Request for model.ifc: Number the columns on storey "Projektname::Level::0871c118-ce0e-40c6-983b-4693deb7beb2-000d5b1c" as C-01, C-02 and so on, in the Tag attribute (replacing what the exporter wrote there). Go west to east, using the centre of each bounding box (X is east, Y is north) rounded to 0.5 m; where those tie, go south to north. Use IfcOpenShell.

First a look at what the model holds.

```python
import ifcopenshell
import ifcopenshell.util.element
import ifcopenshell.util.placement

model = ifcopenshell.open("model.ifc")
print(model.schema)
storey = next(s for s in model.by_type("IfcBuildingStorey") if s.Name == "Projektname::Level::0871c118-ce0e-40c6-983b-4693deb7beb2-000d5b1c")
columns = [e for e in ifcopenshell.util.element.get_decomposition(storey) if e.is_a("IfcColumn")]
for e in sorted(columns, key=lambda e: e.id()):
    origin = ifcopenshell.util.placement.get_local_placement(e.ObjectPlacement)[:3, 3]
    print(e.id(), e.Tag, e.Name, origin.round(2) + 0.0, sep=" | ")
```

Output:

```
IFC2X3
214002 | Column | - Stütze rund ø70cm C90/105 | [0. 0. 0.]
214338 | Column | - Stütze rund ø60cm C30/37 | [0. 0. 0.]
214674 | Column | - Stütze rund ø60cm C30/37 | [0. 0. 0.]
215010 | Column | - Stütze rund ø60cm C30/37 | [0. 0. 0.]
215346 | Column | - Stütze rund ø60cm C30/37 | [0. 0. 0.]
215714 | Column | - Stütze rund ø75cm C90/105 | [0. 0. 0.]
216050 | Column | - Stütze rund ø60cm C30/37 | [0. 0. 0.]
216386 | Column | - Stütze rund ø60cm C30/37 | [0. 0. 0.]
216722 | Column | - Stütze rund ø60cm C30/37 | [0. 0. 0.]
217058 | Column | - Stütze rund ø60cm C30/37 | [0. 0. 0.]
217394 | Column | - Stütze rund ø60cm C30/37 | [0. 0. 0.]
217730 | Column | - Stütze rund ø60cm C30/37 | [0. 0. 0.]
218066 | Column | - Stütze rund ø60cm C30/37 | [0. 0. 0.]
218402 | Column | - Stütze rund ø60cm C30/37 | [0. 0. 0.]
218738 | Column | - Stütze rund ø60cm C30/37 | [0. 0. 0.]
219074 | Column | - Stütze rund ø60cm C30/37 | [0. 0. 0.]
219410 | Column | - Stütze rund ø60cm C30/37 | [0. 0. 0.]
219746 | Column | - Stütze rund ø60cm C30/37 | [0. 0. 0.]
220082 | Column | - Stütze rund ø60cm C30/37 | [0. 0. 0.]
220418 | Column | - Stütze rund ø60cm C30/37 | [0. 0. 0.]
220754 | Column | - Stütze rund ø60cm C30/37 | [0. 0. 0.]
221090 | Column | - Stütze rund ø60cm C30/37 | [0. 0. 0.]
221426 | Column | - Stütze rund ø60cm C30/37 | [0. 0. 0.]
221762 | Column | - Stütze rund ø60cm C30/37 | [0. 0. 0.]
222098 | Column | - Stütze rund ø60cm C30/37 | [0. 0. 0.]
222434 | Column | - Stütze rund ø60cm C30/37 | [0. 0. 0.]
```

```python
import ifcopenshell
import ifcopenshell.geom
import ifcopenshell.util.element
import ifcopenshell.util.shape

model = ifcopenshell.open("model.ifc")
settings = ifcopenshell.geom.settings()
settings.set("use-world-coords", True)


def centre(element):
    shape = ifcopenshell.geom.create_shape(settings, element)
    return ifcopenshell.util.shape.get_bbox_centroid(shape.geometry)


storey = next(s for s in model.by_type("IfcBuildingStorey") if s.Name == "Projektname::Level::0871c118-ce0e-40c6-983b-4693deb7beb2-000d5b1c")
columns = [e for e in ifcopenshell.util.element.get_decomposition(storey) if e.is_a("IfcColumn")]

# Insertion points can sit at a corner or the storey origin, so sort by the geometry (in metres).
centres = {e: centre(e) for e in columns}
columns.sort(key=lambda e: (round(centres[e][0] / 0.5), centres[e][1]))

for i, e in enumerate(columns, start=1):
    number = f"C-{i:02d}"
    e.Tag = number
    print(e.id(), number)

model.write("model_rev.ifc")
```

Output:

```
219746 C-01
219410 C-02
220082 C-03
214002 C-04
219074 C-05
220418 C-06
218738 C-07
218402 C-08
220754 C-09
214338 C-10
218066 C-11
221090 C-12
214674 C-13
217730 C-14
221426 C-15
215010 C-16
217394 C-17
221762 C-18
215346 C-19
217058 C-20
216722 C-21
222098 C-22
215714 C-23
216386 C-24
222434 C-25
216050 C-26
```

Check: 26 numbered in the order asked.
